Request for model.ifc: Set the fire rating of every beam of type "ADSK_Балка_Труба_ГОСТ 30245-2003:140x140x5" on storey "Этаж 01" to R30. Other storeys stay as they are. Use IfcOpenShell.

First a look at what the model holds.

```python
import ifcopenshell
import ifcopenshell.util.element

model = ifcopenshell.open("model.ifc")
print(model.schema)
storey = next(s for s in model.by_type("IfcBuildingStorey") if s.Name == "Этаж 01")
beams = [e for e in ifcopenshell.util.element.get_decomposition(storey) if e.is_a("IfcBeam")]
seen = {}
for e in beams:
    element_type = ifcopenshell.util.element.get_type(e)
    key = (element_type.Name if element_type != e and element_type else None, ifcopenshell.util.element.get_pset(e, "Pset_BeamCommon", "FireRating"))
    seen[key] = seen.get(key, 0) + 1
for (name, value), count in sorted(seen.items(), key=str):
    print(count, "x", name, "|", value)
```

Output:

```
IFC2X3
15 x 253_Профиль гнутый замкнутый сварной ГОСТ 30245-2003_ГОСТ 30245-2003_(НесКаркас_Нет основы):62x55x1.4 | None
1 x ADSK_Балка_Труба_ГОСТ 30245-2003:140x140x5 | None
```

```python
import ifcopenshell
import ifcopenshell.api.pset
import ifcopenshell.util.element

model = ifcopenshell.open("model.ifc")

storey = next(s for s in model.by_type("IfcBuildingStorey") if s.Name == "Этаж 01")
beams = [e for e in ifcopenshell.util.element.get_decomposition(storey) if e.is_a("IfcBeam")]

count = 0
for e in beams:
    element_type = ifcopenshell.util.element.get_type(e)
    if element_type in (None, e) or element_type.Name != "ADSK_Балка_Труба_ГОСТ 30245-2003:140x140x5":
        continue
    # add_pset returns the element's existing set when there is one.
    pset = ifcopenshell.api.pset.add_pset(model, product=e, name="Pset_BeamCommon")
    ifcopenshell.api.pset.edit_pset(model, pset=pset, properties={"FireRating": "R30"})
    count += 1

print(count, "beams updated")

model.write("model_edited.ifc")
```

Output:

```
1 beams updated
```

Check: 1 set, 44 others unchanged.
